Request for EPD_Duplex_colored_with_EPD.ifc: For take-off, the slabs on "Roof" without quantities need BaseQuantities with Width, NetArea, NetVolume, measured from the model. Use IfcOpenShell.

First a look at what the model holds.

```python
import ifcopenshell
import ifcopenshell.util.element
import ifcopenshell.util.unit

model = ifcopenshell.open("EPD_Duplex_colored_with_EPD.ifc")
print(model.schema)
for unit_type in ("LENGTHUNIT", "AREAUNIT", "VOLUMEUNIT"):
    print(unit_type, ifcopenshell.util.unit.calculate_unit_scale(model, unit_type))
storey = next(s for s in model.by_type("IfcBuildingStorey") if s.Name == "Roof")
slabs = [e for e in ifcopenshell.util.element.get_decomposition(storey) if e.is_a("IfcSlab")]
for e in sorted(slabs, key=lambda e: e.id()):
    print(e.id(), e.is_a(), e.Name, list(ifcopenshell.util.element.get_psets(e, qtos_only=True)), sep=" | ")
```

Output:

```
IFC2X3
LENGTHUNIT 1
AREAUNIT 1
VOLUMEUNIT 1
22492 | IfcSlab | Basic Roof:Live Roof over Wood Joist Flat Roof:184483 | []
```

```python
import ifcopenshell
import ifcopenshell.api.pset
import ifcopenshell.geom
import ifcopenshell.util.element
import ifcopenshell.util.shape
import ifcopenshell.util.unit

model = ifcopenshell.open("EPD_Duplex_colored_with_EPD.ifc")
unit_scale = ifcopenshell.util.unit.calculate_unit_scale(model)
area_scale = ifcopenshell.util.unit.calculate_unit_scale(model, "AREAUNIT")
volume_scale = ifcopenshell.util.unit.calculate_unit_scale(model, "VOLUMEUNIT")
settings = ifcopenshell.geom.settings()

storey = next(s for s in model.by_type("IfcBuildingStorey") if s.Name == "Roof")
slabs = [e for e in ifcopenshell.util.element.get_decomposition(storey) if e.is_a("IfcSlab")]

for e in sorted(slabs, key=lambda e: e.id()):
    if ifcopenshell.util.element.get_psets(e, qtos_only=True, should_inherit=False):
        continue
    # Geometry comes back in metres, in the element's own axes.
    shape = ifcopenshell.geom.create_shape(settings, e)
    values = {
        "Width": ifcopenshell.util.shape.get_z(shape.geometry) / unit_scale,
        "NetArea": ifcopenshell.util.shape.get_footprint_area(shape.geometry) / area_scale,
        "NetVolume": ifcopenshell.util.shape.get_volume(shape.geometry) / volume_scale,
    }
    qto = ifcopenshell.api.pset.add_qto(model, product=e, name="BaseQuantities")
    ifcopenshell.api.pset.edit_qto(model, qto=qto, properties=values)
    print(e.id(), {k: round(v, 3) for k, v in values.items()})

model.write("EPD_Duplex_colored_with_EPD_rev.ifc")
```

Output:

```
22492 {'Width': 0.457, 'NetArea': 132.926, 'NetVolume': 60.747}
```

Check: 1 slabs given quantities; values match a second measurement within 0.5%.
